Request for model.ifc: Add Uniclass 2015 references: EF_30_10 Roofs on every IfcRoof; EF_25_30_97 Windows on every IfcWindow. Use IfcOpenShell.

First a look at what the model holds.

```python
import ifcopenshell

model = ifcopenshell.open("model.ifc")
print(model.schema)
print("classifications:", [c.Name for c in model.by_type("IfcClassification")])
for ifc_class in ("IfcDoor", "IfcRoof", "IfcStair", "IfcWall", "IfcWindow"):
    print(ifc_class, len(model.by_type(ifc_class)))
```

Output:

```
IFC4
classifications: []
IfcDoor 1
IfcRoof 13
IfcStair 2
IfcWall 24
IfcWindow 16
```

```python
import ifcopenshell
import ifcopenshell.api.classification

model = ifcopenshell.open("model.ifc")

system = ifcopenshell.api.classification.add_classification(model, classification="Uniclass 2015")

codes = {
    "IfcRoof": ("EF_30_10", "Roofs"),
    "IfcWindow": ("EF_25_30_97", "Windows"),
}
for ifc_class, (code, name) in codes.items():
    products = model.by_type(ifc_class)
    ifcopenshell.api.classification.add_reference(
        model, products=products, classification=system, identification=code, name=name
    )
    print(code, len(products))

model.write("model_edited.ifc")
```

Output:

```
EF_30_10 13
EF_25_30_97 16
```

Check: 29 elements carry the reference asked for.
